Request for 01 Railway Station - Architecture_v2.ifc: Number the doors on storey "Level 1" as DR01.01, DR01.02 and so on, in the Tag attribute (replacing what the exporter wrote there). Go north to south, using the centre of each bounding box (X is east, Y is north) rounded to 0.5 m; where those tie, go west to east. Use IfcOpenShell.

First a look at what the model holds.

```python
import ifcopenshell
import ifcopenshell.util.element
import ifcopenshell.util.placement

model = ifcopenshell.open("01 Railway Station - Architecture_v2.ifc")
print(model.schema)
storey = next(s for s in model.by_type("IfcBuildingStorey") if s.Name == "Level 1")
doors = [e for e in ifcopenshell.util.element.get_decomposition(storey) if e.is_a("IfcDoor")]
for e in sorted(doors, key=lambda e: e.id()):
    origin = ifcopenshell.util.placement.get_local_placement(e.ObjectPlacement)[:3, 3]
    print(e.id(), e.Tag, e.Name, origin.round(2) + 0.0, sep=" | ")
```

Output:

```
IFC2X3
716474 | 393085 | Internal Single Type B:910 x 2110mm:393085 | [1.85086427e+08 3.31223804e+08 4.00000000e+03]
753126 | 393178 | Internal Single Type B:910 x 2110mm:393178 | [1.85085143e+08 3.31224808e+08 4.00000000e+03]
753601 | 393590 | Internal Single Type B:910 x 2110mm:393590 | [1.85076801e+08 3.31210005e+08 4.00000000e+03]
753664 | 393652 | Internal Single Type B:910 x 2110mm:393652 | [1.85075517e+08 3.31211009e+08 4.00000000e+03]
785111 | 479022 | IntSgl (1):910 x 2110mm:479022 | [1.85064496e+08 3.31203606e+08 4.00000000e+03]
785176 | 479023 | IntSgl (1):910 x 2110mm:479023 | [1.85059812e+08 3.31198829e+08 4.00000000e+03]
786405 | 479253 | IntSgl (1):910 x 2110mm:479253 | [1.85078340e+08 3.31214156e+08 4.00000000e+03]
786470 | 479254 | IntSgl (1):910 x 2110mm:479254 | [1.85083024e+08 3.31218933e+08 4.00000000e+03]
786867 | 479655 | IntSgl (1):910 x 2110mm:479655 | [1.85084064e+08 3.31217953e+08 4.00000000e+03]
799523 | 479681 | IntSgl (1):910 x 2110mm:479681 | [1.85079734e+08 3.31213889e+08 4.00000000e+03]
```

```python
import ifcopenshell
import ifcopenshell.geom
import ifcopenshell.util.element
import ifcopenshell.util.shape

model = ifcopenshell.open("01 Railway Station - Architecture_v2.ifc")
settings = ifcopenshell.geom.settings()
settings.set("use-world-coords", True)


def centre(element):
    shape = ifcopenshell.geom.create_shape(settings, element)
    return ifcopenshell.util.shape.get_bbox_centroid(shape.geometry)


storey = next(s for s in model.by_type("IfcBuildingStorey") if s.Name == "Level 1")
doors = [e for e in ifcopenshell.util.element.get_decomposition(storey) if e.is_a("IfcDoor")]

# Insertion points can sit at a corner or the storey origin, so sort by the geometry (in metres).
centres = {e: centre(e) for e in doors}
doors.sort(key=lambda e: (-round(centres[e][1] / 0.5), centres[e][0]))

for i, e in enumerate(doors, start=1):
    number = f"DR01.{i:02d}"
    e.Tag = number
    print(e.id(), number)

model.write("01 Railway Station - Architecture_v2_rev.ifc")
```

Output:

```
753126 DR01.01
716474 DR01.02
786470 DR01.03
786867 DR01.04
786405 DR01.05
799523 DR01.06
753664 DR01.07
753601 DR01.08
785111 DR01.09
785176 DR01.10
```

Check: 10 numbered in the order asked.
